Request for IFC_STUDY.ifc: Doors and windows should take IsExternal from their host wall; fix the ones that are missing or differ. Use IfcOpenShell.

First a look at what the model holds.

```python
import ifcopenshell
import ifcopenshell.util.element

model = ifcopenshell.open("IFC_STUDY.ifc")
print(model.schema)
seen = {}
for e in model.by_type("IfcDoor") + model.by_type("IfcWindow"):
    if not e.FillsVoids:
        continue
    host = e.FillsVoids[0].RelatingOpeningElement.VoidsElements[0].RelatingBuildingElement
    own = ifcopenshell.util.element.get_pset(e, f"Pset_{e.is_a()[3:].removesuffix('StandardCase')}Common", "IsExternal")
    wall = ifcopenshell.util.element.get_pset(host, "Pset_WallCommon", "IsExternal")
    seen[e.is_a(), own, wall] = seen.get((e.is_a(), own, wall), 0) + 1
for (cls, own, wall), count in sorted(seen.items(), key=str):
    print(count, cls, "IsExternal:", own, "| host wall:", wall)
```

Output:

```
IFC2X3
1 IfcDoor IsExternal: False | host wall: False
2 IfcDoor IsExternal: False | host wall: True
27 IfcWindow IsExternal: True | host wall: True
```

```python
import ifcopenshell
import ifcopenshell.api.pset
import ifcopenshell.util.element

model = ifcopenshell.open("IFC_STUDY.ifc")

count = 0
for ifc_class, pset_name in (("IfcDoor", "Pset_DoorCommon"), ("IfcWindow", "Pset_WindowCommon")):
    for e in model.by_type(ifc_class):
        if not e.FillsVoids:
            continue
        host = e.FillsVoids[0].RelatingOpeningElement.VoidsElements[0].RelatingBuildingElement
        external = ifcopenshell.util.element.get_pset(host, "Pset_WallCommon", "IsExternal")
        if external is None or ifcopenshell.util.element.get_pset(e, pset_name, "IsExternal") == external:
            continue
        pset = ifcopenshell.api.pset.add_pset(model, product=e, name=pset_name)
        ifcopenshell.api.pset.edit_pset(model, pset=pset, properties={"IsExternal": external})
        count += 1

print(count, "updated")

model.write("IFC_STUDY-out.ifc")
```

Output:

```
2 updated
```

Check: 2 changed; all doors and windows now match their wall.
